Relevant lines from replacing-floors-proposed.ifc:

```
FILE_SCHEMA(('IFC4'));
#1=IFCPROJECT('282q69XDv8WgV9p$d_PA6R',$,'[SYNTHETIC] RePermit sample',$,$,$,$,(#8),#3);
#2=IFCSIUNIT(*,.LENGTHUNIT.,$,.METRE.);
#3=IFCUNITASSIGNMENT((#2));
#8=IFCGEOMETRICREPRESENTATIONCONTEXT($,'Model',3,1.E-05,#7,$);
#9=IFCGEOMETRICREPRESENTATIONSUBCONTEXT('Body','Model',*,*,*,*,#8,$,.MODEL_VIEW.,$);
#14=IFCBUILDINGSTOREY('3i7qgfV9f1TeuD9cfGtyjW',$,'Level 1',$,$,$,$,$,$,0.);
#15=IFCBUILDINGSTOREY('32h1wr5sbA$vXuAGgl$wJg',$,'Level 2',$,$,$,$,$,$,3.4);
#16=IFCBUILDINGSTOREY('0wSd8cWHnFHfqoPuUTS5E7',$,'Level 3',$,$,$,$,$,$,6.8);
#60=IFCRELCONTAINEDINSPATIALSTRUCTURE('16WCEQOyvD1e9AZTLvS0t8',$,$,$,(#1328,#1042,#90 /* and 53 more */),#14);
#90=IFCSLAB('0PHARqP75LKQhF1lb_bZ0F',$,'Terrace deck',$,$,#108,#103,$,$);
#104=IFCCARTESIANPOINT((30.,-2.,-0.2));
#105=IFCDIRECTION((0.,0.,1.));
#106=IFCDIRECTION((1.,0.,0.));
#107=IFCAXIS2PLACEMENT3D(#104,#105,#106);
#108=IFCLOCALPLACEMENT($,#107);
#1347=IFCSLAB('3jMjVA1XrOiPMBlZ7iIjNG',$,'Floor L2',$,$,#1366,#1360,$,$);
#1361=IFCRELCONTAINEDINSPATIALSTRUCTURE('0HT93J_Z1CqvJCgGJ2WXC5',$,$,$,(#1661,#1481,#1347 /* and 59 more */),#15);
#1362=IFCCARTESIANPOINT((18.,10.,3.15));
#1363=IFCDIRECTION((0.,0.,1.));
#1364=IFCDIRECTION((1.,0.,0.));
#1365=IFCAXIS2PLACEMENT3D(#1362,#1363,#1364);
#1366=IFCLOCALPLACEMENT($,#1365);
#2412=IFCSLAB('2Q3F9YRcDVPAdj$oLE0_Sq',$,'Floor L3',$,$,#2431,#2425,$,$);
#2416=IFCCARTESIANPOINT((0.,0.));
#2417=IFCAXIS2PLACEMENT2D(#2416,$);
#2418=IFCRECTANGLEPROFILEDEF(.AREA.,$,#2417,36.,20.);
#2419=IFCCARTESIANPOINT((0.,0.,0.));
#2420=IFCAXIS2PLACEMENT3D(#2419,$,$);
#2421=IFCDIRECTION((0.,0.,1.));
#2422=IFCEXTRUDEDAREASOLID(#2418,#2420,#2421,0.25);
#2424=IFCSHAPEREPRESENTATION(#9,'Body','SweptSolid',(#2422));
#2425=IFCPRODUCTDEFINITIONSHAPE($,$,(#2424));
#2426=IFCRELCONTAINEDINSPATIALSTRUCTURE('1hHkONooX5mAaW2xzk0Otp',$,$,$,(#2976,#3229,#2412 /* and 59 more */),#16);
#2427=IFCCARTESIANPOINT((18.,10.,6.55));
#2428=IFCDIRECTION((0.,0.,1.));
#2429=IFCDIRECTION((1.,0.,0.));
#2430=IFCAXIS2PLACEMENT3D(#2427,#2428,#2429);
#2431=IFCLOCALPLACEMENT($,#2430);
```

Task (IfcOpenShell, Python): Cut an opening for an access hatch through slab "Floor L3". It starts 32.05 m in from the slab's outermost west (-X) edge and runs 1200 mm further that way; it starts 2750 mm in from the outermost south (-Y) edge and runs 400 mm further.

```python
import numpy as np
import ifcopenshell
import ifcopenshell.api.feature
import ifcopenshell.api.geometry
import ifcopenshell.api.root
import ifcopenshell.geom
import ifcopenshell.util.placement
import ifcopenshell.util.representation
import ifcopenshell.util.shape
import ifcopenshell.util.unit

model = ifcopenshell.open("replacing-floors-proposed.ifc")
unit_scale = ifcopenshell.util.unit.calculate_unit_scale(model)
settings = ifcopenshell.geom.settings()


def volume(element):
    """Net volume in cubic metres, openings subtracted."""
    shape = ifcopenshell.geom.create_shape(settings, element)
    return ifcopenshell.util.shape.get_volume(shape.geometry)


slab = model.by_guid("2Q3F9YRcDVPAdj$oLE0_Sq")
before = volume(slab)

# Extent in the slab's own axes, in metres. The edges named are its -X and -Y sides.
slab_shape = ifcopenshell.geom.create_shape(settings, slab)
vertices = ifcopenshell.util.shape.get_vertices(slab_shape.geometry)
x_min, y_min, bottom = vertices.min(axis=0)
top = vertices[:, 2].max()

opening = ifcopenshell.api.root.create_entity(model, ifc_class="IfcOpeningElement", name="Access hatch opening", predefined_type="OPENING")
context = ifcopenshell.util.representation.get_context(model, "Model", "Body", "MODEL_VIEW")
width, depth = 1.2, 0.4
outline = [(0.0, 0.0), (width, 0.0), (width, depth), (0.0, depth), (0.0, 0.0)]
# Overshoot both faces by 50 mm so the cut is clean.
shape = ifcopenshell.api.geometry.add_slab_representation(
    model, context=context, depth=top - bottom + 0.1, polyline=outline
)
ifcopenshell.api.geometry.assign_representation(model, product=opening, representation=shape)

matrix = ifcopenshell.util.placement.get_local_placement(slab.ObjectPlacement)
matrix[:, 3] = matrix @ np.append(np.array([x_min + 32.05, y_min + 2.75, bottom - 0.05]) / unit_scale, 1.0)
ifcopenshell.api.geometry.edit_object_placement(model, product=opening, matrix=matrix, is_si=False)
ifcopenshell.api.feature.add_feature(model, feature=opening, element=slab)

after = volume(slab)

print(f"slab volume {before:.3f} -> {after:.3f} m3")

model.write("replacing-floors-proposed_updated.ifc")
```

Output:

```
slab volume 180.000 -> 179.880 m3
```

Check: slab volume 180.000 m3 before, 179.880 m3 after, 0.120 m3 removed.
